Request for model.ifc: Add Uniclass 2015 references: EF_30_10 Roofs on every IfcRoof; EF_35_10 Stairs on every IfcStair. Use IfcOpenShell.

First a look at what the model holds.

```python
import ifcopenshell

model = ifcopenshell.open("model.ifc")
print(model.schema)
print("classifications:", [c.Name for c in model.by_type("IfcClassification")])
for ifc_class in ("IfcDoor", "IfcRoof", "IfcStair", "IfcWall", "IfcWindow"):
    print(ifc_class, len(model.by_type(ifc_class)))
```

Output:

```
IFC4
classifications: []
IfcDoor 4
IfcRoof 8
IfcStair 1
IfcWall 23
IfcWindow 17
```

```python
import ifcopenshell
import ifcopenshell.api.classification

model = ifcopenshell.open("model.ifc")

system = ifcopenshell.api.classification.add_classification(model, classification="Uniclass 2015")

codes = {
    "IfcRoof": ("EF_30_10", "Roofs"),
    "IfcStair": ("EF_35_10", "Stairs"),
}
for ifc_class, (code, name) in codes.items():
    products = model.by_type(ifc_class)
    ifcopenshell.api.classification.add_reference(
        model, products=products, classification=system, identification=code, name=name
    )
    print(code, len(products))

model.write("model_rev.ifc")
```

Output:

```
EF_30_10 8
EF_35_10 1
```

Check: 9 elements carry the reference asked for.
